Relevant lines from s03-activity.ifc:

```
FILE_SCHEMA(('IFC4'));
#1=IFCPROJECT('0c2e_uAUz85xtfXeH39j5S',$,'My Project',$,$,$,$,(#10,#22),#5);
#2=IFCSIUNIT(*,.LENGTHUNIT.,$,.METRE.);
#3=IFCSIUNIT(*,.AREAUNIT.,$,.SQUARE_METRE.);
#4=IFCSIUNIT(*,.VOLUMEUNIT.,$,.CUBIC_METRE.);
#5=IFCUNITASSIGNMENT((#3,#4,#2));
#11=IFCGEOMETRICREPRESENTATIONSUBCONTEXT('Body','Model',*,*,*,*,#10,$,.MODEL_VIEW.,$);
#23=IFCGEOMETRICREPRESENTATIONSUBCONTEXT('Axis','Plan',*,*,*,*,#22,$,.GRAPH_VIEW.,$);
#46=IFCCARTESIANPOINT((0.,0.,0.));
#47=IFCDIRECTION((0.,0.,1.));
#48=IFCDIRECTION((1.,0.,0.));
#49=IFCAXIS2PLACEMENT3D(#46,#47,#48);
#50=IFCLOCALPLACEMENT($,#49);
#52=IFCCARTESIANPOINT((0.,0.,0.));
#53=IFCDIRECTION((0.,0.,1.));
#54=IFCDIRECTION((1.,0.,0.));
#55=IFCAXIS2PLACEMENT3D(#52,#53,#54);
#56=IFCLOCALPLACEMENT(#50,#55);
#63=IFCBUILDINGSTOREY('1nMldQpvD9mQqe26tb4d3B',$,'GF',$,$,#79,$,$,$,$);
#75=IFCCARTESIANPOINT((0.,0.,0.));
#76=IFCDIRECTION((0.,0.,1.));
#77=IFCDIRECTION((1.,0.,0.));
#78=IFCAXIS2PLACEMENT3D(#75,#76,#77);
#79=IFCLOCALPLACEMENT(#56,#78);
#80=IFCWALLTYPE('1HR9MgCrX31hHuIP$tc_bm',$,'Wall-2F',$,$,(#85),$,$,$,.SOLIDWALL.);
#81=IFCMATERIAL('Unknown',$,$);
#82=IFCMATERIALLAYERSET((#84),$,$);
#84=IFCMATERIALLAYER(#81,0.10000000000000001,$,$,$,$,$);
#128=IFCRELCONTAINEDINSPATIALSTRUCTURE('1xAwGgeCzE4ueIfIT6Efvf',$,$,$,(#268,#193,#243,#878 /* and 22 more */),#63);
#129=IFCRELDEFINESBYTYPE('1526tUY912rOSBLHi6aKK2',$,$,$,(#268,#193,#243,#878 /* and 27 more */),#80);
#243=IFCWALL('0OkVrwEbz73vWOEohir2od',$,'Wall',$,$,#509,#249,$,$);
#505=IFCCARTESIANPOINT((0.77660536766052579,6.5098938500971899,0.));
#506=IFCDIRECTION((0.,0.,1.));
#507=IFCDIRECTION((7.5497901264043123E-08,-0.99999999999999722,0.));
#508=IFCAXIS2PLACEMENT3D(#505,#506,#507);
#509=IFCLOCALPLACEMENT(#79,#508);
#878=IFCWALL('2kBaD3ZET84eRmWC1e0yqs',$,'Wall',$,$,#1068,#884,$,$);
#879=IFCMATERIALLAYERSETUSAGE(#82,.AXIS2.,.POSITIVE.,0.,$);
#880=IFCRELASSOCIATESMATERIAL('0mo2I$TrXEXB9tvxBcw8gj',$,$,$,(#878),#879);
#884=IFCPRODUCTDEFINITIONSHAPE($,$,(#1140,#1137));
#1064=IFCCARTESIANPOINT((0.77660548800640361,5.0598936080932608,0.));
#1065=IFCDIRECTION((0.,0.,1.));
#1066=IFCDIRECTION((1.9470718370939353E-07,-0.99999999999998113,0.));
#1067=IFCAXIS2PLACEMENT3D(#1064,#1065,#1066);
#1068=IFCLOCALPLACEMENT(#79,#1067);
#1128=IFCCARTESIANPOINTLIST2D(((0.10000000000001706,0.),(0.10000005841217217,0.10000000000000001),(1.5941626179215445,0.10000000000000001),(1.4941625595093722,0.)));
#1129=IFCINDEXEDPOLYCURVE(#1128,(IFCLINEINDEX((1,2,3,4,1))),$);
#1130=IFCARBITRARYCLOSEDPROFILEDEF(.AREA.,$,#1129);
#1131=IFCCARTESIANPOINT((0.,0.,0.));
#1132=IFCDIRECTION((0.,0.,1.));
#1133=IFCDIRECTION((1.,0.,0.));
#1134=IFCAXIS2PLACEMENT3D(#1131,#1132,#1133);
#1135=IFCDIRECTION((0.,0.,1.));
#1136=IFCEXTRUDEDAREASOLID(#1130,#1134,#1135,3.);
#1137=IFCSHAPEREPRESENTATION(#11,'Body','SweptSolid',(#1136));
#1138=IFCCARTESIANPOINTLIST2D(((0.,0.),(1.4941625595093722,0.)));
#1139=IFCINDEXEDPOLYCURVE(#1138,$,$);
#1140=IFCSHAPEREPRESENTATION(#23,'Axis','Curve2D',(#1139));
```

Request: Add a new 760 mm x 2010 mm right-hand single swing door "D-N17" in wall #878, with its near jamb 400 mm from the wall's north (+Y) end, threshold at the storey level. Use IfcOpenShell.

```python
import numpy as np
import ifcopenshell
import ifcopenshell.api.feature
import ifcopenshell.api.geometry
import ifcopenshell.api.root
import ifcopenshell.api.spatial
import ifcopenshell.geom
import ifcopenshell.util.element
import ifcopenshell.util.placement
import ifcopenshell.util.representation
import ifcopenshell.util.shape
import ifcopenshell.util.unit

model = ifcopenshell.open("s03-activity.ifc")
unit_scale = ifcopenshell.util.unit.calculate_unit_scale(model)
settings = ifcopenshell.geom.settings()


def volume(element):
    """Net volume in cubic metres, openings subtracted."""
    shape = ifcopenshell.geom.create_shape(settings, element)
    return ifcopenshell.util.shape.get_volume(shape.geometry)


wall = model.by_guid("2kBaD3ZET84eRmWC1e0yqs")
storey = ifcopenshell.util.element.get_container(wall, ifc_class="IfcBuildingStorey")
context = ifcopenshell.util.representation.get_context(model, "Model", "Body", "MODEL_VIEW")
before = volume(wall)

width, height, from_end, sill = 0.76, 2.01, 0.4, 0.0  # metres

# The wall runs along its own X axis, and the end named is its -X end.
wall_shape = ifcopenshell.geom.create_shape(settings, wall)
x, y, z = ifcopenshell.util.shape.get_vertices(wall_shape.geometry).T
start = x.min() + from_end
face, thickness = float(y.min()), float(y.max() - y.min())
wall_matrix = ifcopenshell.util.placement.get_local_placement(wall.ObjectPlacement)
level = ifcopenshell.util.placement.get_local_placement(storey.ObjectPlacement)[2, 3]


def in_wall(x, y):
    """Placement at x, y metres in the wall's axes, at sill height."""
    matrix = wall_matrix.copy()
    matrix[:, 3] = wall_matrix @ np.array([x / unit_scale, y / unit_scale, 0.0, 1.0])
    matrix[2, 3] = level + sill / unit_scale
    return matrix


# Opening: a box that overshoots both wall faces by 50 mm.
opening = ifcopenshell.api.root.create_entity(model, ifc_class="IfcOpeningElement", predefined_type="OPENING")
box = ifcopenshell.api.geometry.add_wall_representation(
    model, context=context, length=width, height=height, thickness=thickness + 0.1
)
ifcopenshell.api.geometry.assign_representation(model, product=opening, representation=box)
ifcopenshell.api.geometry.edit_object_placement(model, product=opening, matrix=in_wall(start, face - 0.05), is_si=False)
ifcopenshell.api.feature.add_feature(model, feature=opening, element=wall)

door = ifcopenshell.api.root.create_entity(model, ifc_class="IfcDoor", name="D-N17", predefined_type="DOOR")
door.OverallWidth, door.OverallHeight = width / unit_scale, height / unit_scale
door.OperationType = "SINGLE_SWING_RIGHT"
body = ifcopenshell.api.geometry.add_door_representation(
    model,
    context=context,
    overall_width=door.OverallWidth,
    overall_height=door.OverallHeight,
    operation_type="SINGLE_SWING_RIGHT",
    lining_properties={"LiningDepth": thickness / unit_scale, "ThresholdDepth": thickness / unit_scale},
)
ifcopenshell.api.geometry.assign_representation(model, product=door, representation=body)
ifcopenshell.api.spatial.assign_container(model, products=[door], relating_structure=storey)
ifcopenshell.api.feature.add_filling(model, opening=opening, element=door)

# The lining spans the wall, so the door starts at the wall face.
ifcopenshell.api.geometry.edit_object_placement(model, product=door, matrix=in_wall(start, face), is_si=False)

after = volume(wall)

print(f"wall volume {before:.3f} -> {after:.3f} m3")

model.write("s03-activity_v2.ifc")
```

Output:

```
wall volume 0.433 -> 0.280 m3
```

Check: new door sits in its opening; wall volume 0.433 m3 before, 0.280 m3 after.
